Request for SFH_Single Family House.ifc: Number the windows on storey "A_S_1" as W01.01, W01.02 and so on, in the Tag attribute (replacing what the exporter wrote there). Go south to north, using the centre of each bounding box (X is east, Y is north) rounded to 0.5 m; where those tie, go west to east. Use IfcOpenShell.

First a look at what the model holds.

```python
import ifcopenshell
import ifcopenshell.util.element
import ifcopenshell.util.placement

model = ifcopenshell.open("SFH_Single Family House.ifc")
print(model.schema)
storey = next(s for s in model.by_type("IfcBuildingStorey") if s.Name == "A_S_1")
windows = [e for e in ifcopenshell.util.element.get_decomposition(storey) if e.is_a("IfcWindow")]
for e in sorted(windows, key=lambda e: e.id()):
    origin = ifcopenshell.util.placement.get_local_placement(e.ObjectPlacement)[:3, 3]
    print(e.id(), e.Tag, e.Name, origin.round(2) + 0.0, sep=" | ")
```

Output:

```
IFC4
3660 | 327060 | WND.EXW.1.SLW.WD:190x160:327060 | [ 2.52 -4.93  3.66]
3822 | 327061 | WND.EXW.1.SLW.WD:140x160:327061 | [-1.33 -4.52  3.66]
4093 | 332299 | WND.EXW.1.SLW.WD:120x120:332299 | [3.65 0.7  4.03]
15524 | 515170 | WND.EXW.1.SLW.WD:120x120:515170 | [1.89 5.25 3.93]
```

```python
import ifcopenshell
import ifcopenshell.geom
import ifcopenshell.util.element
import ifcopenshell.util.shape

model = ifcopenshell.open("SFH_Single Family House.ifc")
settings = ifcopenshell.geom.settings()
settings.set("use-world-coords", True)


def centre(element):
    shape = ifcopenshell.geom.create_shape(settings, element)
    return ifcopenshell.util.shape.get_bbox_centroid(shape.geometry)


storey = next(s for s in model.by_type("IfcBuildingStorey") if s.Name == "A_S_1")
windows = [e for e in ifcopenshell.util.element.get_decomposition(storey) if e.is_a("IfcWindow")]

# Insertion points can sit at a corner or the storey origin, so sort by the geometry (in metres).
centres = {e: centre(e) for e in windows}
windows.sort(key=lambda e: (round(centres[e][1] / 0.5), centres[e][0]))

for i, e in enumerate(windows, start=1):
    number = f"W01.{i:02d}"
    e.Tag = number
    print(e.id(), number)

model.write("SFH_Single Family House_edited.ifc")
```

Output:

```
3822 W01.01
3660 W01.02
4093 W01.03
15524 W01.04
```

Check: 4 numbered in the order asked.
